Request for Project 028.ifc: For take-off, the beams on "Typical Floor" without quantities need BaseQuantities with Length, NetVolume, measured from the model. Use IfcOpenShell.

First a look at what the model holds.

```python
import ifcopenshell
import ifcopenshell.util.element
import ifcopenshell.util.unit

model = ifcopenshell.open("Project 028.ifc")
print(model.schema)
for unit_type in ("LENGTHUNIT", "AREAUNIT", "VOLUMEUNIT"):
    print(unit_type, ifcopenshell.util.unit.calculate_unit_scale(model, unit_type))
storey = next(s for s in model.by_type("IfcBuildingStorey") if s.Name == "Typical Floor")
beams = [e for e in ifcopenshell.util.element.get_decomposition(storey) if e.is_a("IfcBeam")]
for e in sorted(beams, key=lambda e: e.id()):
    print(e.id(), e.is_a(), e.Name, list(ifcopenshell.util.element.get_psets(e, qtos_only=True)), sep=" | ")
```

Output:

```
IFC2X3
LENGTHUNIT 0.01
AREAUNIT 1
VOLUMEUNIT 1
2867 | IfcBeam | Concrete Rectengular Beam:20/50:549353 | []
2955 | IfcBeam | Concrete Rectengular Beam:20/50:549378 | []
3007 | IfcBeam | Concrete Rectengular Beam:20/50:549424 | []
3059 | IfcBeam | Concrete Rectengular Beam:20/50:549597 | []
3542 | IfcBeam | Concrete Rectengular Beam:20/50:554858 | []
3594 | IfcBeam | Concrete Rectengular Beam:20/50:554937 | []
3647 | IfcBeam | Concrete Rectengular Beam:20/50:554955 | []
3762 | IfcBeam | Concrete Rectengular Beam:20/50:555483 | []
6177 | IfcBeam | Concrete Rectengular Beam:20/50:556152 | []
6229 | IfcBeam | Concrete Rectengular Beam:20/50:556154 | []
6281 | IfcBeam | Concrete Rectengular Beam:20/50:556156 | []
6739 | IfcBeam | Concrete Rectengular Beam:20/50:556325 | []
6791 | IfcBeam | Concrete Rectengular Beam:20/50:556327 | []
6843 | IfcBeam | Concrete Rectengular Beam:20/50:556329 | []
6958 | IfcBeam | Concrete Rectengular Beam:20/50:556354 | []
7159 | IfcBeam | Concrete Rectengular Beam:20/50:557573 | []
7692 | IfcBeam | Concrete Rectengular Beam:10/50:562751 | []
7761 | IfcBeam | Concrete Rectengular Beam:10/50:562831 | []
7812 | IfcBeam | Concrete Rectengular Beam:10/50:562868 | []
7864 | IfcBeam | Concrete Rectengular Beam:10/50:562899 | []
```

```python
import ifcopenshell
import ifcopenshell.api.pset
import ifcopenshell.geom
import ifcopenshell.util.element
import ifcopenshell.util.shape
import ifcopenshell.util.unit

model = ifcopenshell.open("Project 028.ifc")
unit_scale = ifcopenshell.util.unit.calculate_unit_scale(model)
volume_scale = ifcopenshell.util.unit.calculate_unit_scale(model, "VOLUMEUNIT")
settings = ifcopenshell.geom.settings()

storey = next(s for s in model.by_type("IfcBuildingStorey") if s.Name == "Typical Floor")
beams = [e for e in ifcopenshell.util.element.get_decomposition(storey) if e.is_a("IfcBeam")]

for e in sorted(beams, key=lambda e: e.id()):
    if ifcopenshell.util.element.get_psets(e, qtos_only=True, should_inherit=False):
        continue
    # Geometry comes back in metres, in the element's own axes.
    shape = ifcopenshell.geom.create_shape(settings, e)
    values = {
        "Length": ifcopenshell.util.shape.get_max_xyz(shape.geometry) / unit_scale,
        "NetVolume": ifcopenshell.util.shape.get_volume(shape.geometry) / volume_scale,
    }
    qto = ifcopenshell.api.pset.add_qto(model, product=e, name="BaseQuantities")
    ifcopenshell.api.pset.edit_qto(model, qto=qto, properties=values)
    print(e.id(), {k: round(v, 3) for k, v in values.items()})

model.write("Project 028_updated.ifc")
```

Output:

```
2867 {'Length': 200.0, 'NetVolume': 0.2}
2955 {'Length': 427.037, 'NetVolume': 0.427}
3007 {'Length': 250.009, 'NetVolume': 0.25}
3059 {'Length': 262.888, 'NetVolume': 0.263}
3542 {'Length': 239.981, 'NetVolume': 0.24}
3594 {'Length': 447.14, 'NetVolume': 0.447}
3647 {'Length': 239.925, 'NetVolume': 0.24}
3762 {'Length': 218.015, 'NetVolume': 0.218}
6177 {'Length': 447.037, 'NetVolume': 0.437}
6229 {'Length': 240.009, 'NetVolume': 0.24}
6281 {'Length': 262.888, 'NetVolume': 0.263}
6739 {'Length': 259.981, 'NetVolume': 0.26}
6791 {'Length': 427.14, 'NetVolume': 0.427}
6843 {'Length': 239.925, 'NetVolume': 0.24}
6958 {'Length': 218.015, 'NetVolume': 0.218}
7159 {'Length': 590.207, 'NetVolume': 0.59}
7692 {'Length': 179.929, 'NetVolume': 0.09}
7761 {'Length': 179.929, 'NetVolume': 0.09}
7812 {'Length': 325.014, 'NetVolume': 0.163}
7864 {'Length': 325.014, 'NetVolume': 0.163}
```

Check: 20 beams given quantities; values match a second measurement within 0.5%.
